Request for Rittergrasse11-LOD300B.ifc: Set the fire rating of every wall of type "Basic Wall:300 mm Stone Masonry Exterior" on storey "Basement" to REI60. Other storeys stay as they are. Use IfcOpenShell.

First a look at what the model holds.

```python
import ifcopenshell
import ifcopenshell.util.element

model = ifcopenshell.open("Rittergrasse11-LOD300B.ifc")
print(model.schema)
storey = next(s for s in model.by_type("IfcBuildingStorey") if s.Name == "Basement")
walls = [e for e in ifcopenshell.util.element.get_decomposition(storey) if e.is_a("IfcWall")]
seen = {}
for e in walls:
    element_type = ifcopenshell.util.element.get_type(e)
    key = (element_type.Name if element_type != e and element_type else None, ifcopenshell.util.element.get_pset(e, "Pset_WallCommon", "FireRating"))
    seen[key] = seen.get(key, 0) + 1
for (name, value), count in sorted(seen.items(), key=str):
    print(count, "x", name, "|", value)
```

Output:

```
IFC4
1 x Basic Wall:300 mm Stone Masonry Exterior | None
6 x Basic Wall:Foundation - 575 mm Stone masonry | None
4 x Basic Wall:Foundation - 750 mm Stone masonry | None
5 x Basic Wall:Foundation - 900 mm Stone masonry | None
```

```python
import ifcopenshell
import ifcopenshell.api.pset
import ifcopenshell.util.element

model = ifcopenshell.open("Rittergrasse11-LOD300B.ifc")

storey = next(s for s in model.by_type("IfcBuildingStorey") if s.Name == "Basement")
walls = [e for e in ifcopenshell.util.element.get_decomposition(storey) if e.is_a("IfcWall")]

count = 0
for e in walls:
    element_type = ifcopenshell.util.element.get_type(e)
    if element_type in (None, e) or element_type.Name != "Basic Wall:300 mm Stone Masonry Exterior":
        continue
    # add_pset returns the element's existing set when there is one.
    pset = ifcopenshell.api.pset.add_pset(model, product=e, name="Pset_WallCommon")
    ifcopenshell.api.pset.edit_pset(model, pset=pset, properties={"FireRating": "REI60"})
    count += 1

print(count, "walls updated")

model.write("Rittergrasse11-LOD300B-out.ifc")
```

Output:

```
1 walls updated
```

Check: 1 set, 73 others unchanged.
